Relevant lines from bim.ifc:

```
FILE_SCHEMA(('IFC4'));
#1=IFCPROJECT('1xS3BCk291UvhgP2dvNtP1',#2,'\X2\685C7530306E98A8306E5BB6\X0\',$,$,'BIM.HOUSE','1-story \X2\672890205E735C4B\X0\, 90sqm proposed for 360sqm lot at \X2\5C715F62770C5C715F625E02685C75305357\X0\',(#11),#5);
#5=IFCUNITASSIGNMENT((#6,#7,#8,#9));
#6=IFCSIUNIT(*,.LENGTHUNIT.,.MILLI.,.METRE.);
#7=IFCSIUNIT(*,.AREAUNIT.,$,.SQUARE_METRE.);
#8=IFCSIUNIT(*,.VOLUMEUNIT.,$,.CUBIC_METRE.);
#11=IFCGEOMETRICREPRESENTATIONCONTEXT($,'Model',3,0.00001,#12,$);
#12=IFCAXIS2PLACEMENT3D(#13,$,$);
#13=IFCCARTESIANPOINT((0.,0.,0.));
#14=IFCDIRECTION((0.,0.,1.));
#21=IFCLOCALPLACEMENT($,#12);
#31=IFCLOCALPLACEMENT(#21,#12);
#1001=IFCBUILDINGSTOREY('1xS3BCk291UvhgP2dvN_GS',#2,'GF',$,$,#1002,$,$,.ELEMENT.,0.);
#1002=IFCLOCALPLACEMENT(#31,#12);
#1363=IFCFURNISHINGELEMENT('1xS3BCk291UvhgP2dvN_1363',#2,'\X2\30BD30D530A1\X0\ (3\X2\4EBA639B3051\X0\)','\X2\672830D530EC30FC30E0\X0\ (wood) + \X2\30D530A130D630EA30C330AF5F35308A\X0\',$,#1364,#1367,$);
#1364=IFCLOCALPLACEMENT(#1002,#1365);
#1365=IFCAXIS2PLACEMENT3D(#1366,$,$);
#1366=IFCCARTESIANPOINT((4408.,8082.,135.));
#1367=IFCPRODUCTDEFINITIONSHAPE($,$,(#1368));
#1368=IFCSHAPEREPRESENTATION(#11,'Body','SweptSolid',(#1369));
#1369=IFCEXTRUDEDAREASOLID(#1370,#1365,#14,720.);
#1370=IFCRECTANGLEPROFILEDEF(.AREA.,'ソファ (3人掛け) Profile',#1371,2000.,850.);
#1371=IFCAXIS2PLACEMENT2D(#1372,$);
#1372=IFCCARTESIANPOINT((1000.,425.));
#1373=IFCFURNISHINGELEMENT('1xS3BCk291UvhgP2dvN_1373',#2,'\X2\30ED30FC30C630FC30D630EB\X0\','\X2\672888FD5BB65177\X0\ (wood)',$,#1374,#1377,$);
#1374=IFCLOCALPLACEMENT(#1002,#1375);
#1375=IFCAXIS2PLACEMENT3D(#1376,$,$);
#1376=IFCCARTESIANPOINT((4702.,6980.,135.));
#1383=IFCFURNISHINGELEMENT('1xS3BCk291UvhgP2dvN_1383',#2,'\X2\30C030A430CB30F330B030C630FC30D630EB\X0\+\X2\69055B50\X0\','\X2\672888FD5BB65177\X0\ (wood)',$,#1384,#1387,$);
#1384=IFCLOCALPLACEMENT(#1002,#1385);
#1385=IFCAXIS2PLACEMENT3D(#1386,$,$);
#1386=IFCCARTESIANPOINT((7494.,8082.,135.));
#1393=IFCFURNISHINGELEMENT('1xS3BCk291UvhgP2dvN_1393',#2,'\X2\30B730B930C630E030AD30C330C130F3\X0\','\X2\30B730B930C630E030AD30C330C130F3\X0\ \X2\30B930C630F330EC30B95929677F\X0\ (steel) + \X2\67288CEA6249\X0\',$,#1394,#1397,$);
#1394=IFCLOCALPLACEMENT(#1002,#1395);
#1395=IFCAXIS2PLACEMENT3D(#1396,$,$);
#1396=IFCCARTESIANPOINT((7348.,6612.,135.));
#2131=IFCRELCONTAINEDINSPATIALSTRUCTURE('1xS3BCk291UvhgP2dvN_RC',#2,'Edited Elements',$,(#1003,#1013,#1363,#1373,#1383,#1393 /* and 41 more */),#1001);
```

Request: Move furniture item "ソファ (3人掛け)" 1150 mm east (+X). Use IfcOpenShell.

```python
import ifcopenshell
import ifcopenshell.api.geometry
import ifcopenshell.util.placement

model = ifcopenshell.open("bim.ifc")

item = model.by_guid("1xS3BCk291UvhgP2dvN_1363")
matrix = ifcopenshell.util.placement.get_local_placement(item.ObjectPlacement)
matrix[0, 3] += 1150.0
ifcopenshell.api.geometry.edit_object_placement(model, product=item, matrix=matrix, is_si=False)

print(ifcopenshell.util.placement.get_local_placement(item.ObjectPlacement).round(3) + 0.0)

model.write("bim_rev.ifc")
```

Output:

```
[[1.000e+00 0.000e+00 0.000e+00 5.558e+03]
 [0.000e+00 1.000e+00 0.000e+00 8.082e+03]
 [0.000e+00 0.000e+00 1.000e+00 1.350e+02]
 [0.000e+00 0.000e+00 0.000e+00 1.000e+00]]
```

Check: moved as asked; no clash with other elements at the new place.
